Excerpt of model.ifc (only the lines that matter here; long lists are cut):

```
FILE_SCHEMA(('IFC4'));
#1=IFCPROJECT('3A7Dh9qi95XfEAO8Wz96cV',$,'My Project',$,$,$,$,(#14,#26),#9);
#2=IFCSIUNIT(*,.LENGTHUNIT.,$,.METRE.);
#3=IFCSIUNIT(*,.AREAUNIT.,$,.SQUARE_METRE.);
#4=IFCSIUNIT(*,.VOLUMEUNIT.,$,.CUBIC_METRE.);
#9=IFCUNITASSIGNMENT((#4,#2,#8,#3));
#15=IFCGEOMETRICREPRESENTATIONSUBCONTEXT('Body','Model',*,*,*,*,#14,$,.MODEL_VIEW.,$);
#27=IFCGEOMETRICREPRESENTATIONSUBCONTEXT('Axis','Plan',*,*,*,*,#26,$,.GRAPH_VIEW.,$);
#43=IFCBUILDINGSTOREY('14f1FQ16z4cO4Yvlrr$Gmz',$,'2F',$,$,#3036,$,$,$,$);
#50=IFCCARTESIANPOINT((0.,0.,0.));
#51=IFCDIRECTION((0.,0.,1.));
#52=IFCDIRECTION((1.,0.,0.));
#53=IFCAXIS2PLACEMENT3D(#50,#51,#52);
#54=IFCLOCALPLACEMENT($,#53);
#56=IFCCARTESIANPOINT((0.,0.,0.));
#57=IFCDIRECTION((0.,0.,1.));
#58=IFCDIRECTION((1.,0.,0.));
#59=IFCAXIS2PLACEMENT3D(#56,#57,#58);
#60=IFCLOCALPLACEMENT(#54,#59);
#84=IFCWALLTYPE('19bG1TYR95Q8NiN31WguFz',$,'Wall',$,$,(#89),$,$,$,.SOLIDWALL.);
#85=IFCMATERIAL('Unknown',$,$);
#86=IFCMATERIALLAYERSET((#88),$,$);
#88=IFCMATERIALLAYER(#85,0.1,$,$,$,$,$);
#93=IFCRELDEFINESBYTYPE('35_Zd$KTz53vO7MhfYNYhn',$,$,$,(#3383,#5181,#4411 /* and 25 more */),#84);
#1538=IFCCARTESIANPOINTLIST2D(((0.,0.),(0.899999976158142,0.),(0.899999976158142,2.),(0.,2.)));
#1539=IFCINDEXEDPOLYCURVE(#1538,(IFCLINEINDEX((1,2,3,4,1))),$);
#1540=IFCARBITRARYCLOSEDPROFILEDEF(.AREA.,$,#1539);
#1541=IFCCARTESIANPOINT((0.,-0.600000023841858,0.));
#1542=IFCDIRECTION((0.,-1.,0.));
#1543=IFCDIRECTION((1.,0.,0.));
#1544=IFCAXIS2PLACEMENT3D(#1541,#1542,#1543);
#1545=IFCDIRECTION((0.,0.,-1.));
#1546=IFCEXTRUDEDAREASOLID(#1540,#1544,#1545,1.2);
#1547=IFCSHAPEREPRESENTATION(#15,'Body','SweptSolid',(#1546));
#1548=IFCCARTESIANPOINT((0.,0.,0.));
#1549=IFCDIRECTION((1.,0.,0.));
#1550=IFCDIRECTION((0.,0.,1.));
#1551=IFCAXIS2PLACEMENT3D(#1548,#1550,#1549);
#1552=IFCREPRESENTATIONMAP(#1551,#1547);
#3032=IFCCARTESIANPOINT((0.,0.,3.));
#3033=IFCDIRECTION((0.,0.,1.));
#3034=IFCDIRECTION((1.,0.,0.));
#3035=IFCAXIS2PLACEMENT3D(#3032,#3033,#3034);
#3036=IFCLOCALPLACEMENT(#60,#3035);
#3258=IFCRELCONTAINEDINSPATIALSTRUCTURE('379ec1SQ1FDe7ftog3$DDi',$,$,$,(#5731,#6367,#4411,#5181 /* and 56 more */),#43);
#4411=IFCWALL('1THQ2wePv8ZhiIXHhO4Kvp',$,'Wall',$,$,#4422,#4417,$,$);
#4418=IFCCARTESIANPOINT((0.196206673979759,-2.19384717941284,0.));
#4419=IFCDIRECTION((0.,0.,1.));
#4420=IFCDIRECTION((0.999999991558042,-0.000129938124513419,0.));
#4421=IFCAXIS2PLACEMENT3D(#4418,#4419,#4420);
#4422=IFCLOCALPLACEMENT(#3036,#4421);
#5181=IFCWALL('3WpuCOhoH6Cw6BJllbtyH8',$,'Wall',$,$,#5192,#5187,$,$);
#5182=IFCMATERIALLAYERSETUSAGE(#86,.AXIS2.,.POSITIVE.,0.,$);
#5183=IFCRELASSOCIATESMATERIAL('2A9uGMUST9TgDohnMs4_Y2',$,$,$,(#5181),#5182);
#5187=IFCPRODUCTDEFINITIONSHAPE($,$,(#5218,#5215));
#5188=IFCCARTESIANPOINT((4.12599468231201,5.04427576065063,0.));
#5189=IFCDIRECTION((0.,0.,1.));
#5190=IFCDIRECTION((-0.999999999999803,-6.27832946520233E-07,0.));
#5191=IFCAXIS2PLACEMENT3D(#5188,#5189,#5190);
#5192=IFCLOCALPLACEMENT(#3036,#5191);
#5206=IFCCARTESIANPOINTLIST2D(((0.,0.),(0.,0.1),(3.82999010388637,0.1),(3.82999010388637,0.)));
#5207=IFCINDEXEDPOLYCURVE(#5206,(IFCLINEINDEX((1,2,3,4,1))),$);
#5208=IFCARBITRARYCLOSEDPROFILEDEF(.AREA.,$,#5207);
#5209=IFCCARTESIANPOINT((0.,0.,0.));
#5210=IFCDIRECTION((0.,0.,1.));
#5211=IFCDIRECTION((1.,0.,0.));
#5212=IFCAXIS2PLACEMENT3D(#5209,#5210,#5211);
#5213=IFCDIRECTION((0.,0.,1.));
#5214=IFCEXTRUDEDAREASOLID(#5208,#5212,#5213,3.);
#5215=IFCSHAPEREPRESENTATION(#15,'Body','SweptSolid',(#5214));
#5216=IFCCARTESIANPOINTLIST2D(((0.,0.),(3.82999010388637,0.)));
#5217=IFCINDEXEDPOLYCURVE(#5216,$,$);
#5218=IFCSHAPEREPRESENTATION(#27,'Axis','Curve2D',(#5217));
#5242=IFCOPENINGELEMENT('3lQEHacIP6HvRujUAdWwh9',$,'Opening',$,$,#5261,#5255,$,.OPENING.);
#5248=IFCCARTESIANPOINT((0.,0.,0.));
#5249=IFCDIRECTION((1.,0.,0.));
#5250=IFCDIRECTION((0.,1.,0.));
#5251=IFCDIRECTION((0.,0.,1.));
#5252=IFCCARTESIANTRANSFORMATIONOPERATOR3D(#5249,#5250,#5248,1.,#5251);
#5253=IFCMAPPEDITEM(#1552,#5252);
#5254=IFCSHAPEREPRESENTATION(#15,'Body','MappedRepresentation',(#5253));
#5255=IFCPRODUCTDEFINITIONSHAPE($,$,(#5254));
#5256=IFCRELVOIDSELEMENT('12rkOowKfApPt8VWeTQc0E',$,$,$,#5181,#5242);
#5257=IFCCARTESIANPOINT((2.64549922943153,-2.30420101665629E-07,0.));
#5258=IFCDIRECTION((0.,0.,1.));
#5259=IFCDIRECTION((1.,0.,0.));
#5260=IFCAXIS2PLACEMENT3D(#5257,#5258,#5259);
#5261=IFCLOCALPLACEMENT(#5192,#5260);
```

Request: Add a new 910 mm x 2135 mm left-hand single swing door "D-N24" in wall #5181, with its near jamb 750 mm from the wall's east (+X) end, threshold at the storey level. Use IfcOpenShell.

```python
import numpy as np
import ifcopenshell
import ifcopenshell.api.feature
import ifcopenshell.api.geometry
import ifcopenshell.api.root
import ifcopenshell.api.spatial
import ifcopenshell.geom
import ifcopenshell.util.element
import ifcopenshell.util.placement
import ifcopenshell.util.representation
import ifcopenshell.util.shape
import ifcopenshell.util.unit

model = ifcopenshell.open("model.ifc")
unit_scale = ifcopenshell.util.unit.calculate_unit_scale(model)
settings = ifcopenshell.geom.settings()


def volume(element):
    """Net volume in cubic metres, openings subtracted."""
    shape = ifcopenshell.geom.create_shape(settings, element)
    return ifcopenshell.util.shape.get_volume(shape.geometry)


wall = model.by_guid("3WpuCOhoH6Cw6BJllbtyH8")
storey = ifcopenshell.util.element.get_container(wall, ifc_class="IfcBuildingStorey")
context = ifcopenshell.util.representation.get_context(model, "Model", "Body", "MODEL_VIEW")
before = volume(wall)

width, height, from_end, sill = 0.91, 2.135, 0.75, 0.0  # metres

# The wall runs along its own X axis, and the end named is its -X end.
wall_shape = ifcopenshell.geom.create_shape(settings, wall)
x, y, z = ifcopenshell.util.shape.get_vertices(wall_shape.geometry).T
start = x.min() + from_end
face, thickness = float(y.min()), float(y.max() - y.min())
wall_matrix = ifcopenshell.util.placement.get_local_placement(wall.ObjectPlacement)
level = ifcopenshell.util.placement.get_local_placement(storey.ObjectPlacement)[2, 3]


def in_wall(x, y):
    """Placement at x, y metres in the wall's axes, at sill height."""
    matrix = wall_matrix.copy()
    matrix[:, 3] = wall_matrix @ np.array([x / unit_scale, y / unit_scale, 0.0, 1.0])
    matrix[2, 3] = level + sill / unit_scale
    return matrix


# Opening: a box that overshoots both wall faces by 50 mm.
opening = ifcopenshell.api.root.create_entity(model, ifc_class="IfcOpeningElement", predefined_type="OPENING")
box = ifcopenshell.api.geometry.add_wall_representation(
    model, context=context, length=width, height=height, thickness=thickness + 0.1
)
ifcopenshell.api.geometry.assign_representation(model, product=opening, representation=box)
ifcopenshell.api.geometry.edit_object_placement(model, product=opening, matrix=in_wall(start, face - 0.05), is_si=False)
ifcopenshell.api.feature.add_feature(model, feature=opening, element=wall)

door = ifcopenshell.api.root.create_entity(model, ifc_class="IfcDoor", name="D-N24", predefined_type="DOOR")
door.OverallWidth, door.OverallHeight = width / unit_scale, height / unit_scale
door.OperationType = "SINGLE_SWING_LEFT"
body = ifcopenshell.api.geometry.add_door_representation(
    model,
    context=context,
    overall_width=door.OverallWidth,
    overall_height=door.OverallHeight,
    operation_type="SINGLE_SWING_LEFT",
    lining_properties={"LiningDepth": thickness / unit_scale, "ThresholdDepth": thickness / unit_scale},
)
ifcopenshell.api.geometry.assign_representation(model, product=door, representation=body)
ifcopenshell.api.spatial.assign_container(model, products=[door], relating_structure=storey)
ifcopenshell.api.feature.add_filling(model, opening=opening, element=door)

# The lining spans the wall, so the door starts at the wall face.
ifcopenshell.api.geometry.edit_object_placement(model, product=door, matrix=in_wall(start, face), is_si=False)

after = volume(wall)

print(f"wall volume {before:.3f} -> {after:.3f} m3")

model.write("model_rev.ifc")
```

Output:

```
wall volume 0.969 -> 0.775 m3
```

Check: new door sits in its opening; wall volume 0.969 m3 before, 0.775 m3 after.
